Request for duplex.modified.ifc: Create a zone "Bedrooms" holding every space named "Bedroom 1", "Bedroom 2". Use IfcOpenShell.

First a look at what the model holds.

```python
import ifcopenshell

model = ifcopenshell.open("duplex.modified.ifc")
print(model.schema)
seen = {}
for space in model.by_type("IfcSpace"):
    seen[space.LongName] = seen.get(space.LongName, 0) + 1
for name, count in sorted(seen.items(), key=str):
    print(count, "x", name)
print("zones:", [z.Name for z in model.by_type("IfcZone")][:20])
```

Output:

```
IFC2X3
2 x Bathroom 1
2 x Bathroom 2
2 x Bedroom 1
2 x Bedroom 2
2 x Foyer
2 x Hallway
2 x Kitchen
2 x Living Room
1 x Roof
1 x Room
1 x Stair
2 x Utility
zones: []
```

```python
import ifcopenshell
import ifcopenshell.api.group
import ifcopenshell.api.root

model = ifcopenshell.open("duplex.modified.ifc")

names = {"Bedroom 1", "Bedroom 2"}
spaces = [s for s in model.by_type("IfcSpace") if s.LongName in names]

zone = ifcopenshell.api.root.create_entity(model, ifc_class="IfcZone", name="Bedrooms")
ifcopenshell.api.group.assign_group(model, products=spaces, group=zone)
print(len(spaces), "spaces in", zone.Name)

model.write("duplex.modified_edited.ifc")
```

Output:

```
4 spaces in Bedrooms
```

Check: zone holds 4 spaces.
